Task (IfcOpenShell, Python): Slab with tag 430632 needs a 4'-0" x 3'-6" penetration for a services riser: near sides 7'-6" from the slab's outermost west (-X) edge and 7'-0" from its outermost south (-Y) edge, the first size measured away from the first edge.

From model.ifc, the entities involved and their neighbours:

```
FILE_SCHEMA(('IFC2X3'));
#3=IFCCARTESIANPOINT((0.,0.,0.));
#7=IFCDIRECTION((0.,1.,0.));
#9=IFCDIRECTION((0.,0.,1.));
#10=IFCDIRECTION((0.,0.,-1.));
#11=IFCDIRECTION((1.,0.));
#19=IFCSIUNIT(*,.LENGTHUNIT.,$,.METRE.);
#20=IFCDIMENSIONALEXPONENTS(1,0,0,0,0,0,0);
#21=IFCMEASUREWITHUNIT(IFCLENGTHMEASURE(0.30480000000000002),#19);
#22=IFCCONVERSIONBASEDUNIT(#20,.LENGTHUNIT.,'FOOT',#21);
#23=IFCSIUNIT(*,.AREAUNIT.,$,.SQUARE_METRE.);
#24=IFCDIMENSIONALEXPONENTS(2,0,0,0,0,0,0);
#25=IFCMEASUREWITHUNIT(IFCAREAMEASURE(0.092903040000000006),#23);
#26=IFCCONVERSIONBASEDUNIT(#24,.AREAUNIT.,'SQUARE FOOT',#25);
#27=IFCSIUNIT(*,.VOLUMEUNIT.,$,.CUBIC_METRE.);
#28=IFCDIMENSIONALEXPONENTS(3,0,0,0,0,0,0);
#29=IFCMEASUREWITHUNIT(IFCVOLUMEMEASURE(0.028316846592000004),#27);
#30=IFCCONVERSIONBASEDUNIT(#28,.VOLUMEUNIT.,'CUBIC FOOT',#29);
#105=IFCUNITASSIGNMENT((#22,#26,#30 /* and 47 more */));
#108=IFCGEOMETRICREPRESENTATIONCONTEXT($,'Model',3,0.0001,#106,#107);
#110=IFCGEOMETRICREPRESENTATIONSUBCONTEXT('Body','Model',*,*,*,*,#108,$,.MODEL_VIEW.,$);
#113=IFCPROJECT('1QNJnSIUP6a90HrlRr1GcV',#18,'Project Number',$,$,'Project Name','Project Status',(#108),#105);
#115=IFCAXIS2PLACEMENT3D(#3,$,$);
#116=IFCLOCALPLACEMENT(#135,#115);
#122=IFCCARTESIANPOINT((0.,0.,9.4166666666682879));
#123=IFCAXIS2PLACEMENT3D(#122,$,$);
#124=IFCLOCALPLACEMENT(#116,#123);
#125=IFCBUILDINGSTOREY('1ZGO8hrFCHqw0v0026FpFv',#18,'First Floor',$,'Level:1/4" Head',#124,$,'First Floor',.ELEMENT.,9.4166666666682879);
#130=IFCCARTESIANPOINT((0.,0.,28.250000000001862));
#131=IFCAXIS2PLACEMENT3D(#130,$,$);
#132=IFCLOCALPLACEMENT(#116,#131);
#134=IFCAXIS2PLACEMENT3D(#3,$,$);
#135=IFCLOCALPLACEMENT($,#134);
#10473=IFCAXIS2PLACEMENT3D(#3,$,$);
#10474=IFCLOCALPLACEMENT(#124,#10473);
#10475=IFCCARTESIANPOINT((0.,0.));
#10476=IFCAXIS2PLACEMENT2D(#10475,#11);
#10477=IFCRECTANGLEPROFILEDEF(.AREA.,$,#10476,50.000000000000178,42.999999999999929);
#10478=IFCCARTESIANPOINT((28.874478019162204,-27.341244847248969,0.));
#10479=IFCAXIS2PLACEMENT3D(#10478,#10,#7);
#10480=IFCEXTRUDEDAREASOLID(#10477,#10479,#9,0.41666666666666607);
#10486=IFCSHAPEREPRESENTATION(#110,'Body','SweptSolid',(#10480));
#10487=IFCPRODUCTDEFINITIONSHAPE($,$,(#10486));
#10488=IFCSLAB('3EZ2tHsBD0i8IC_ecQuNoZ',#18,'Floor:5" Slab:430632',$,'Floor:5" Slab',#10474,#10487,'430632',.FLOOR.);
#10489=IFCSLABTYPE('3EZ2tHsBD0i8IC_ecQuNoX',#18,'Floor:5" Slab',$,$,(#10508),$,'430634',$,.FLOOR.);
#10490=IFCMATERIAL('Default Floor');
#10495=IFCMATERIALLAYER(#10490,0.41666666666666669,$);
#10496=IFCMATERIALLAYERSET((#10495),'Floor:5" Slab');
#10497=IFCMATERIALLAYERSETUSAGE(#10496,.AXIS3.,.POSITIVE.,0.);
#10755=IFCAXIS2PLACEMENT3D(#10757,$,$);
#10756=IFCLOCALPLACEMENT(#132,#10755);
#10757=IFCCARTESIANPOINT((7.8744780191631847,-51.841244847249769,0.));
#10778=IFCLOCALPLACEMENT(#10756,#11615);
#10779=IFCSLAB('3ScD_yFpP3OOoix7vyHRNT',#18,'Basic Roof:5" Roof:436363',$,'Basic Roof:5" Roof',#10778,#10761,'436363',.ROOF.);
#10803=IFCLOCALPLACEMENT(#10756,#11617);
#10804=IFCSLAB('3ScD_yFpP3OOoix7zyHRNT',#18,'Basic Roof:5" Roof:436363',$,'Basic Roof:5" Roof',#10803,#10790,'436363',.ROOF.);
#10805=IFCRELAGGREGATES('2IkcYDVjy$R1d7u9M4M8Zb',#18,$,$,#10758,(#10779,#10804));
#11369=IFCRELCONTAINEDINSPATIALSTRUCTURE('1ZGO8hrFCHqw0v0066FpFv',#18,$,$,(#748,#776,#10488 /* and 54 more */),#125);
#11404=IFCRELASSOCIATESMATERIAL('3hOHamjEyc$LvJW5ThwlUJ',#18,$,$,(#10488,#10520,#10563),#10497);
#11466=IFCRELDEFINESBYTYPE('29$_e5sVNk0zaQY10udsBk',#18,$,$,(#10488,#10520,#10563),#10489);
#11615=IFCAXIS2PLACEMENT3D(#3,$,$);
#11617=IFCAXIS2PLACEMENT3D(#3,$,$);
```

```python
import numpy as np
import ifcopenshell
import ifcopenshell.api.feature
import ifcopenshell.api.geometry
import ifcopenshell.api.root
import ifcopenshell.geom
import ifcopenshell.util.placement
import ifcopenshell.util.representation
import ifcopenshell.util.shape
import ifcopenshell.util.unit

model = ifcopenshell.open("model.ifc")
unit_scale = ifcopenshell.util.unit.calculate_unit_scale(model)
settings = ifcopenshell.geom.settings()


def volume(element):
    """Net volume in cubic metres, openings subtracted."""
    shape = ifcopenshell.geom.create_shape(settings, element)
    return ifcopenshell.util.shape.get_volume(shape.geometry)


slab = model.by_guid("3EZ2tHsBD0i8IC_ecQuNoZ")
before = volume(slab)

# Extent in the slab's own axes, in metres. The edges named are its -X and -Y sides.
slab_shape = ifcopenshell.geom.create_shape(settings, slab)
vertices = ifcopenshell.util.shape.get_vertices(slab_shape.geometry)
x_min, y_min, bottom = vertices.min(axis=0)
top = vertices[:, 2].max()

opening = ifcopenshell.api.root.create_entity(model, ifc_class="IfcOpeningElement", name="Services riser opening")
context = ifcopenshell.util.representation.get_context(model, "Model", "Body", "MODEL_VIEW")
width, depth = 1.2192, 1.0668
outline = [(0.0, 0.0), (width, 0.0), (width, depth), (0.0, depth), (0.0, 0.0)]
# Overshoot both faces by 50 mm so the cut is clean.
shape = ifcopenshell.api.geometry.add_slab_representation(
    model, context=context, depth=top - bottom + 0.1, polyline=outline
)
ifcopenshell.api.geometry.assign_representation(model, product=opening, representation=shape)

matrix = ifcopenshell.util.placement.get_local_placement(slab.ObjectPlacement)
matrix[:, 3] = matrix @ np.append(np.array([x_min + 2.286, y_min + 2.1336, bottom - 0.05]) / unit_scale, 1.0)
ifcopenshell.api.geometry.edit_object_placement(model, product=opening, matrix=matrix, is_si=False)
ifcopenshell.api.feature.add_feature(model, feature=opening, element=slab)

after = volume(slab)

print(f"slab volume {before:.3f} -> {after:.3f} m3")

model.write("model-out.ifc")
```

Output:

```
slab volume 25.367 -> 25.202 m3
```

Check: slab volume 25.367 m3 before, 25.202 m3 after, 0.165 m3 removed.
